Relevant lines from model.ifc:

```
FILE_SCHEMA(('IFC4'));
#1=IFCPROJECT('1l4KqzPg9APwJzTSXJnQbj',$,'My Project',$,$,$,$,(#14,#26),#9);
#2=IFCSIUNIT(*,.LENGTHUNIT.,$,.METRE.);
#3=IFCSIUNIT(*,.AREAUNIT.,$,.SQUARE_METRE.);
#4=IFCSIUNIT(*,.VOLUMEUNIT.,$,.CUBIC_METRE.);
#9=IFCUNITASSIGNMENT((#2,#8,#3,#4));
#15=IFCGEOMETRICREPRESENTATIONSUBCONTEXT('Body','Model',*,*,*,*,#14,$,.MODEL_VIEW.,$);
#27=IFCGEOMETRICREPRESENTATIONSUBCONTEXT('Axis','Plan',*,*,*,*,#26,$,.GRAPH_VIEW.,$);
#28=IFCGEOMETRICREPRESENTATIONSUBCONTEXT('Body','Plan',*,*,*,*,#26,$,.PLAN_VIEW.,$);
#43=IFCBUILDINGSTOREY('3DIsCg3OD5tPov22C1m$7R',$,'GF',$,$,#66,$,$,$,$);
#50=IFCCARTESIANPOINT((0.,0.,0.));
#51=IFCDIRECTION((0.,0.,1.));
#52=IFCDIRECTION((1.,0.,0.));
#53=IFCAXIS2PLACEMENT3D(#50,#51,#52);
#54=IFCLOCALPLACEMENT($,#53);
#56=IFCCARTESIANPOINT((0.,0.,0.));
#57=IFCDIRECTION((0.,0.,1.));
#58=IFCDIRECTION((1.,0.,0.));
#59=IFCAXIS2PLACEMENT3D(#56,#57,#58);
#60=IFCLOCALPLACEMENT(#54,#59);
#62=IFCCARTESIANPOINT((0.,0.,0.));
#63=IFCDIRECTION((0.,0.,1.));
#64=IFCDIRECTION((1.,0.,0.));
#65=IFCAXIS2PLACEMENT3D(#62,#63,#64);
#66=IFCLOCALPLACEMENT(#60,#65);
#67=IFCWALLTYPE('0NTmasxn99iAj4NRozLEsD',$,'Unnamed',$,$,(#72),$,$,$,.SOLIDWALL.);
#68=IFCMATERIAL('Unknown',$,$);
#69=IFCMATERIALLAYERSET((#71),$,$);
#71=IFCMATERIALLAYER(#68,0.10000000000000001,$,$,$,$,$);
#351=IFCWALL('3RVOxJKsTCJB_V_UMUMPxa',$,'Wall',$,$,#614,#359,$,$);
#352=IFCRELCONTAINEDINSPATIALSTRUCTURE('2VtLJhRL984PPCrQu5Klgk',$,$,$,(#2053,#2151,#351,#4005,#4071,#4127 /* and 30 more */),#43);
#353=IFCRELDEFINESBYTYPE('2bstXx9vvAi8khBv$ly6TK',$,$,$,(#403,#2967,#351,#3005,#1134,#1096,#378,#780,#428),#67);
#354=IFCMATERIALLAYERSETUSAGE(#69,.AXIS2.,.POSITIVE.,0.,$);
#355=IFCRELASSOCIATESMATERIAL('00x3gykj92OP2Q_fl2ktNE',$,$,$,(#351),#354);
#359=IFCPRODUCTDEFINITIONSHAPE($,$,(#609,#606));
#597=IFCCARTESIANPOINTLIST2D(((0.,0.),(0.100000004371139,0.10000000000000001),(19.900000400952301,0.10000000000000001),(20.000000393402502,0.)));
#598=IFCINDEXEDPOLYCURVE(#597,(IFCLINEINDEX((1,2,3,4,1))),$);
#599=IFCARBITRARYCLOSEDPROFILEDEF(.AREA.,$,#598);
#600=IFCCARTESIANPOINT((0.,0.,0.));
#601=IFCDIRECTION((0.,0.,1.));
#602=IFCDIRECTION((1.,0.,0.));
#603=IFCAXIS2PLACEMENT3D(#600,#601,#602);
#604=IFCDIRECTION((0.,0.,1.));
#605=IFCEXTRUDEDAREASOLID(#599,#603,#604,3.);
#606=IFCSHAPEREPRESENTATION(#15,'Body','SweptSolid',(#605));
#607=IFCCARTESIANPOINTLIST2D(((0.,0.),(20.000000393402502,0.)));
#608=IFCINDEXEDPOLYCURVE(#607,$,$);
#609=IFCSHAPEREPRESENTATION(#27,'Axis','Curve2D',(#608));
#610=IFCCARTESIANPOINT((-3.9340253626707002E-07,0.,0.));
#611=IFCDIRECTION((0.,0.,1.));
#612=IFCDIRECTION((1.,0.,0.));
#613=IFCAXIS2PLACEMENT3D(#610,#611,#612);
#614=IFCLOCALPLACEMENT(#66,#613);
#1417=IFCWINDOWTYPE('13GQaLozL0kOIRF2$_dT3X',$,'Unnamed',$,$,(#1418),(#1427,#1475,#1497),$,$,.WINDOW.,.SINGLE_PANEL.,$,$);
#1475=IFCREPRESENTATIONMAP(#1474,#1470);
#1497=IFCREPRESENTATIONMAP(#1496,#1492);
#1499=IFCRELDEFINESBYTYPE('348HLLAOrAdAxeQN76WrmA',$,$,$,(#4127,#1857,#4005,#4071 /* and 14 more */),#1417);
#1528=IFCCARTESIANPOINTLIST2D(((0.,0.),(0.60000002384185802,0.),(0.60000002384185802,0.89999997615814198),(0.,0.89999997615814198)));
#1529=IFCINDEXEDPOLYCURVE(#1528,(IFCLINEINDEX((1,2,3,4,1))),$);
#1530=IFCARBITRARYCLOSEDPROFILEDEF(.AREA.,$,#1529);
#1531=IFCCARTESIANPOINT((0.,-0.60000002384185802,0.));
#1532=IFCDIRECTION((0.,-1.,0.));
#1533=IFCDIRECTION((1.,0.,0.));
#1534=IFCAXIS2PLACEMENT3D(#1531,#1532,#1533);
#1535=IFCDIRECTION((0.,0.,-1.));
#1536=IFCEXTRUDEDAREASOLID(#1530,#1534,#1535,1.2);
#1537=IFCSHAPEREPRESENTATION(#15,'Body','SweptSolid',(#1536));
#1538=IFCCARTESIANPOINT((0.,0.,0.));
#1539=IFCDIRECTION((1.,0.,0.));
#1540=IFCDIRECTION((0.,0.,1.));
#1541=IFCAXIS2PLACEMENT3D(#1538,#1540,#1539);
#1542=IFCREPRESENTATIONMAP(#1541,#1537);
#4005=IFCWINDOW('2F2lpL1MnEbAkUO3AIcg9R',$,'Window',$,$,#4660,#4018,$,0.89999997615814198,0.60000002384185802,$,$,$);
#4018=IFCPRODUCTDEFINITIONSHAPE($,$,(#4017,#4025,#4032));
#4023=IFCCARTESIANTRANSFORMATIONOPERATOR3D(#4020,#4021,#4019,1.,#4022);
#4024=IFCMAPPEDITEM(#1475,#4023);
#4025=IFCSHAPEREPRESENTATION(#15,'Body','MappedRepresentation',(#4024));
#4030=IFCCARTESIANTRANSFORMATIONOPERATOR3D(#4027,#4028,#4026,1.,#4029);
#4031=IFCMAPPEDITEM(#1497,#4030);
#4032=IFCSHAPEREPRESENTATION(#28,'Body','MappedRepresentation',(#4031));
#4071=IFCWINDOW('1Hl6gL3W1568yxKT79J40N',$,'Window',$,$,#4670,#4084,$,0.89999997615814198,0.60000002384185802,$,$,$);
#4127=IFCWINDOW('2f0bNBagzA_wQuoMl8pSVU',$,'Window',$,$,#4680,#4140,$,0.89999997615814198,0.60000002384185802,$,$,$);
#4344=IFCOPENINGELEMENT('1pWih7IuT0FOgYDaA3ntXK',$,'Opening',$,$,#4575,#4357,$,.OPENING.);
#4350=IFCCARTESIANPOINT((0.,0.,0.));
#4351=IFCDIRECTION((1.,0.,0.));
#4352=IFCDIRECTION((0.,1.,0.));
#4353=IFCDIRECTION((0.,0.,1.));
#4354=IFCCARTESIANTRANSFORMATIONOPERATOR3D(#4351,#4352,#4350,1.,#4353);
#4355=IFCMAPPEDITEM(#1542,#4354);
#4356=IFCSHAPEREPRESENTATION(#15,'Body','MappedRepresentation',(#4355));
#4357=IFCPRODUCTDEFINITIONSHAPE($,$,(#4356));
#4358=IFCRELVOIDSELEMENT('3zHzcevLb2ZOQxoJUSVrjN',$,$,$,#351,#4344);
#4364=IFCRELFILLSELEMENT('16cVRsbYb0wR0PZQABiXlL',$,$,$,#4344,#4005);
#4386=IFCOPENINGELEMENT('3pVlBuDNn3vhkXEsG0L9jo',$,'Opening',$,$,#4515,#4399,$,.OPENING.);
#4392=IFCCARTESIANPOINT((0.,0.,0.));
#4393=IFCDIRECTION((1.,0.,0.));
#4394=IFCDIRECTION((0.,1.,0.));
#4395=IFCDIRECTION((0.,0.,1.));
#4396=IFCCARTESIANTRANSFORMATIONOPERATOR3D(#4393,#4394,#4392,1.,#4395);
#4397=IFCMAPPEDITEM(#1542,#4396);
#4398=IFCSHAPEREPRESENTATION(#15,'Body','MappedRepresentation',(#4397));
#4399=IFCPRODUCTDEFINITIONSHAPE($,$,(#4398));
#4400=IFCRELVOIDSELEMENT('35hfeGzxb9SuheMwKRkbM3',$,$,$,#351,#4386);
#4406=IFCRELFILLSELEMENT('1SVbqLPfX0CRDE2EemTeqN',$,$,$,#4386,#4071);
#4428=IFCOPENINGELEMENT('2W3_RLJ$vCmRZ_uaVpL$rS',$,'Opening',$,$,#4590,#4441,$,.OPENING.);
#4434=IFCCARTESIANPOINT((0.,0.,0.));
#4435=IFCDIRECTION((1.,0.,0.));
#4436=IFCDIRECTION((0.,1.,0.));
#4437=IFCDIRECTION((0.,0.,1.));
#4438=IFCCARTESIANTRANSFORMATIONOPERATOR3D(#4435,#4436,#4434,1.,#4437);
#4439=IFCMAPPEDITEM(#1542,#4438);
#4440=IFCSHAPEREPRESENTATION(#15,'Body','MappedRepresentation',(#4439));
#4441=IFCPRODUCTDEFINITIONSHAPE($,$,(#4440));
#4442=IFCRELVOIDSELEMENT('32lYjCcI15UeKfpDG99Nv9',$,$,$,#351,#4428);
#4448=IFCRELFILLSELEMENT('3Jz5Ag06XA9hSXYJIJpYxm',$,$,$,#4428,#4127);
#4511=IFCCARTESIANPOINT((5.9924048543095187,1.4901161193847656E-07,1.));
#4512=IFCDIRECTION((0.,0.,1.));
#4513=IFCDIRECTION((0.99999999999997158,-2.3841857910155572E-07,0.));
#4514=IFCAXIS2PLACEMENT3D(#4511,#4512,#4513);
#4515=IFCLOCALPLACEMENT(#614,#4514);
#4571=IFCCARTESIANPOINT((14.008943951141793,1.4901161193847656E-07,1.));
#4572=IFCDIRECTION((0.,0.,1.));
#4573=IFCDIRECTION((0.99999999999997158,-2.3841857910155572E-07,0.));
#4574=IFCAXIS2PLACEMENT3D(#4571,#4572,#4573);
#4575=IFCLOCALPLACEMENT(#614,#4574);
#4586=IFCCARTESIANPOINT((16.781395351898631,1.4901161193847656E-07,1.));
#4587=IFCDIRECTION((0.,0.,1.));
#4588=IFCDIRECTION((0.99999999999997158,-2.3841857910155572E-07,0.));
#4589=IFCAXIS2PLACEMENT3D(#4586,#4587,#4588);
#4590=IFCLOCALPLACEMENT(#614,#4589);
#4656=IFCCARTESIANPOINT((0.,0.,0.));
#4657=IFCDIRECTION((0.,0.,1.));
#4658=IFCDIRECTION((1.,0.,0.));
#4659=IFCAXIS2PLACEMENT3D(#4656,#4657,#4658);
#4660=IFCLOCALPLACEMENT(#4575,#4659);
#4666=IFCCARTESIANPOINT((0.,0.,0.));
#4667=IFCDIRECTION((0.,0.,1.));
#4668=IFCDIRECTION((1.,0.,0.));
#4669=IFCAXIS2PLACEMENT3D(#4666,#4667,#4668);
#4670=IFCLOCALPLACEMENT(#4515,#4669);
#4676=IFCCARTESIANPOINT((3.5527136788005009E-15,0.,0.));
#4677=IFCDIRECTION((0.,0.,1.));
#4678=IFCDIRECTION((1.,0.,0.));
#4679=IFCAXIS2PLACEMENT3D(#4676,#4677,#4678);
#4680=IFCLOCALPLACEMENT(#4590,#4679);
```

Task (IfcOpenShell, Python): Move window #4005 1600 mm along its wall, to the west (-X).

```python
import ifcopenshell
import ifcopenshell.api.geometry
import ifcopenshell.util.placement
import ifcopenshell.util.unit

model = ifcopenshell.open("model.ifc")
unit_scale = ifcopenshell.util.unit.calculate_unit_scale(model)

window = model.by_guid("2F2lpL1MnEbAkUO3AIcg9R")
opening = window.FillsVoids[0].RelatingOpeningElement
wall = opening.VoidsElements[0].RelatingBuildingElement

wall_matrix = ifcopenshell.util.placement.get_local_placement(wall.ObjectPlacement)
shift = wall_matrix[:3, 0] * -1.6 / unit_scale
before = ifcopenshell.util.placement.get_local_placement(window.ObjectPlacement)[:3, 3].copy()

# The window is placed relative to its opening, so it follows when the opening moves.
matrix = ifcopenshell.util.placement.get_local_placement(opening.ObjectPlacement)
matrix[:3, 3] += shift
ifcopenshell.api.geometry.edit_object_placement(
    model, product=opening, matrix=matrix, is_si=False, should_transform_children=True
)

after = ifcopenshell.util.placement.get_local_placement(window.ObjectPlacement)[:3, 3]
print("window moved by", (after - before).round(3) + 0.0)

model.write("model_v2.ifc")
```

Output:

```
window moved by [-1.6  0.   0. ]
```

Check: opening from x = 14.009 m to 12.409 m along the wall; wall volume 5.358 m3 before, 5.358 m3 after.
